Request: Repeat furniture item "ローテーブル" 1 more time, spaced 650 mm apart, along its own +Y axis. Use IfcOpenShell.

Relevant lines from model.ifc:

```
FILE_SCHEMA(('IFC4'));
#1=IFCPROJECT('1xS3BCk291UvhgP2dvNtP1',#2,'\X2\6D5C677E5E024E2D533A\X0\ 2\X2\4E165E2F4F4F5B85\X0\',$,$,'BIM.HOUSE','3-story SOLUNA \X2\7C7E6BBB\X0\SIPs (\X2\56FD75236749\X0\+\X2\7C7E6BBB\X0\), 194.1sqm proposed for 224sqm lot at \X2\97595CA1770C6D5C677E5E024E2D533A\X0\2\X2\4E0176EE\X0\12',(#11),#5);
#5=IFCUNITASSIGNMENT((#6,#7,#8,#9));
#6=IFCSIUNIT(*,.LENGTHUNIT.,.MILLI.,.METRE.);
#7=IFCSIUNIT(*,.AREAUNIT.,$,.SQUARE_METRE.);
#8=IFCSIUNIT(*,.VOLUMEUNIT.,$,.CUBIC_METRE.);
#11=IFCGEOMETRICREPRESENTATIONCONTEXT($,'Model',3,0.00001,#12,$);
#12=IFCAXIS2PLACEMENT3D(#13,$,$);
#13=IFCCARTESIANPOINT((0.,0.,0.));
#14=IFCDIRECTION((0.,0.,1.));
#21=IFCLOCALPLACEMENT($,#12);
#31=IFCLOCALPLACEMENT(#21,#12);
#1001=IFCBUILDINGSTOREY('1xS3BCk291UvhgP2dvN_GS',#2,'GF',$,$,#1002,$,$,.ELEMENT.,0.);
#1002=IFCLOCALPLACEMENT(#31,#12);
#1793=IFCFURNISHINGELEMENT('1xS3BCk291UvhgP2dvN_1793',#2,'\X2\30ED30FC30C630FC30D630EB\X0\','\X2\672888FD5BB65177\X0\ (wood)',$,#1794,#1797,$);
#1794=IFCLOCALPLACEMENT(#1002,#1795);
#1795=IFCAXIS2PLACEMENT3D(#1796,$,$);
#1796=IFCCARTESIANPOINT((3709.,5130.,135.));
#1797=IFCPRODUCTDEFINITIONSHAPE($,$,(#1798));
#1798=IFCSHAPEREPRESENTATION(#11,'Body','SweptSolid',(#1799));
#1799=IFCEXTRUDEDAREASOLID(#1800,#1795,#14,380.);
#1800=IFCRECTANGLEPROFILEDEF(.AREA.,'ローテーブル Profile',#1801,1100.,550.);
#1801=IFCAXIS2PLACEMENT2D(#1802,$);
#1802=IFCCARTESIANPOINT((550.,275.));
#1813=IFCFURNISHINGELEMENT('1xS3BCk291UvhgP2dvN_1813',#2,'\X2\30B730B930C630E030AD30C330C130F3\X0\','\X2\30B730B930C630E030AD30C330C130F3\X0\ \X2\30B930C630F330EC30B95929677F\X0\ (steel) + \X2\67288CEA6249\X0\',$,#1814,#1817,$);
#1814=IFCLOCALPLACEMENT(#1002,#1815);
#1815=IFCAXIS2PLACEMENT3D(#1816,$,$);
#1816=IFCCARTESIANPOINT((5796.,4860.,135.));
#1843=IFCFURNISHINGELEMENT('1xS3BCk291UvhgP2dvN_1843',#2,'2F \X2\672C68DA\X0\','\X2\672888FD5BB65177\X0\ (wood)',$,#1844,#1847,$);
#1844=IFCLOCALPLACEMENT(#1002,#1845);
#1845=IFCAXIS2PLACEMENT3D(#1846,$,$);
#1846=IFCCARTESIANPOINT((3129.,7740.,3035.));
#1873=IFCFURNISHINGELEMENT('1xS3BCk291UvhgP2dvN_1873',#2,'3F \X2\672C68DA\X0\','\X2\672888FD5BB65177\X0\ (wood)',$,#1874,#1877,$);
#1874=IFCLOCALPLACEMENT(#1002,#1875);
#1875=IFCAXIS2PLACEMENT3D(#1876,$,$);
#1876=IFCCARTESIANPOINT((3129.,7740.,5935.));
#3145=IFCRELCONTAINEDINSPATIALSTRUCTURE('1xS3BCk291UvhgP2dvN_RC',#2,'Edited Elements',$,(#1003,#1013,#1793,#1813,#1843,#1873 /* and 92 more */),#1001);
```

```python
import ifcopenshell
import ifcopenshell.api.geometry
import ifcopenshell.api.root
import ifcopenshell.util.element
import ifcopenshell.util.placement

model = ifcopenshell.open("model.ifc")


def reuse_history(source, copy):
    """copy_class also copies each property set's owner history, people and application; keep the originals."""
    for rel in copy.IsDefinedBy:
        if rel.is_a("IfcRelDefinesByProperties") and (history := rel.RelatingPropertyDefinition.OwnerHistory):
            rel.RelatingPropertyDefinition.OwnerHistory = source.OwnerHistory
            ifcopenshell.util.element.remove_deep2(model, history)


source = model.by_guid("1xS3BCk291UvhgP2dvN_1793")
base = ifcopenshell.util.placement.get_local_placement(source.ObjectPlacement)
step = base[:3, 1] * 650.0

for i in range(1, 2):
    copy = ifcopenshell.api.root.copy_class(model, product=source)
    copy.Representation = ifcopenshell.util.element.copy_deep(
        model, source.Representation, exclude=["IfcGeometricRepresentationContext", "IfcRepresentationMap"]
    )
    reuse_history(source, copy)
    matrix = base.copy()
    matrix[:3, 3] += i * step
    print("added at", matrix[:3, 3].round(3) + 0.0)
    ifcopenshell.api.geometry.edit_object_placement(model, product=copy, matrix=matrix, is_si=False)

model.write("model-out.ifc")
```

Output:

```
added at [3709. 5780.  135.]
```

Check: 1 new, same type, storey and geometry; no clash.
